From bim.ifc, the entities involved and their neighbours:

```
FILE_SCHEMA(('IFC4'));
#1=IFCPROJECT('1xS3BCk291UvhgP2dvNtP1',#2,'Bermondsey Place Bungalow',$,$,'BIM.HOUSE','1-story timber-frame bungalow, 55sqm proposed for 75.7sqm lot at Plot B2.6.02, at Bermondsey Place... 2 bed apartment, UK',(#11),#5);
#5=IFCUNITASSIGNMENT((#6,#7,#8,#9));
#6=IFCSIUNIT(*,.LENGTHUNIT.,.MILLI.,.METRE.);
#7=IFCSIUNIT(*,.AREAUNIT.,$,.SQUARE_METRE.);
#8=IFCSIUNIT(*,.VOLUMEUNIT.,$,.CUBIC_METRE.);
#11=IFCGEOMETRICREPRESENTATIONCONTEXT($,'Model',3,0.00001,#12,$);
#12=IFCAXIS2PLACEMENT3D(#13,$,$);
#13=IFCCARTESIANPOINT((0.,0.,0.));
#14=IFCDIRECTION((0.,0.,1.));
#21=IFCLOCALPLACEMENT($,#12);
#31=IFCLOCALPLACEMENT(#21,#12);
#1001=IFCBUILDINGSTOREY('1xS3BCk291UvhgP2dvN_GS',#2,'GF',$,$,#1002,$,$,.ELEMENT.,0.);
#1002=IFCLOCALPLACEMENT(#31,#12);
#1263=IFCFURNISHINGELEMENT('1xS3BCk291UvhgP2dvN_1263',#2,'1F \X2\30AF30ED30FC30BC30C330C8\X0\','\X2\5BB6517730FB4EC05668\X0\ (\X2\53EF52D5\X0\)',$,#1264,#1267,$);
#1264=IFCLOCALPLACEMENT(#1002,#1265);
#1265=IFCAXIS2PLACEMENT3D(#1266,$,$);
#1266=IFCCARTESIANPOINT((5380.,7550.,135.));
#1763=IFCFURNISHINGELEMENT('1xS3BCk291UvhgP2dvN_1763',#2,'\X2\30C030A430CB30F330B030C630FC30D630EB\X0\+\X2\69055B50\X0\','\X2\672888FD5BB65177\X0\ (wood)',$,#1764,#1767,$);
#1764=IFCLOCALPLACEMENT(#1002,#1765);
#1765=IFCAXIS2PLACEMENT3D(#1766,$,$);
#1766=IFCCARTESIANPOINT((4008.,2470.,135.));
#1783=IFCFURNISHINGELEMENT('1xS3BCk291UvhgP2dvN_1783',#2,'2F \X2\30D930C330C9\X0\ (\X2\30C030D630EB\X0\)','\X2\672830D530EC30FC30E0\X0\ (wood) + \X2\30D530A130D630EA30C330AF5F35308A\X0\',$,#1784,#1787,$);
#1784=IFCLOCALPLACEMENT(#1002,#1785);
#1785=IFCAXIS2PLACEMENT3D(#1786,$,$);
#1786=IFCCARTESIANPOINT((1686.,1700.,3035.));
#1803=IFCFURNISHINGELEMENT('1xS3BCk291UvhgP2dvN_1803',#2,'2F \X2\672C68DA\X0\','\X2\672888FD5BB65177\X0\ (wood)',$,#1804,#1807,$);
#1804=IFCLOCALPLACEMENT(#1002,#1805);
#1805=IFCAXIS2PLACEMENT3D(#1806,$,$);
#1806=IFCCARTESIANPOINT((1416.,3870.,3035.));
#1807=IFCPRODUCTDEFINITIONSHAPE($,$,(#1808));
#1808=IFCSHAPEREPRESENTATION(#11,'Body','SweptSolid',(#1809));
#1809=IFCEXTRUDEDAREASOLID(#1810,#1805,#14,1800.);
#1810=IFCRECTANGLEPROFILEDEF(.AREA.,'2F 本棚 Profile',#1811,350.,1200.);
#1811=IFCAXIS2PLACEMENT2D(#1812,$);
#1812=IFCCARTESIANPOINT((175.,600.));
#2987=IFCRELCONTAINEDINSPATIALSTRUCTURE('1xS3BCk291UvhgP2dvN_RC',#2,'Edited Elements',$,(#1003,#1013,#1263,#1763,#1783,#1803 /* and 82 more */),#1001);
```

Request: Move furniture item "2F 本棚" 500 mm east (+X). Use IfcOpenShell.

```python
import ifcopenshell
import ifcopenshell.api.geometry
import ifcopenshell.util.placement
import ifcopenshell.util.unit

model = ifcopenshell.open("bim.ifc")
unit_scale = ifcopenshell.util.unit.calculate_unit_scale(model)

item = model.by_id(1803)
matrix = ifcopenshell.util.placement.get_local_placement(item.ObjectPlacement)
matrix[0, 3] += 0.5 / unit_scale
ifcopenshell.api.geometry.edit_object_placement(model, product=item, matrix=matrix, is_si=False)

print(ifcopenshell.util.placement.get_local_placement(item.ObjectPlacement).round(3) + 0.0)

model.write("bim_rev.ifc")
```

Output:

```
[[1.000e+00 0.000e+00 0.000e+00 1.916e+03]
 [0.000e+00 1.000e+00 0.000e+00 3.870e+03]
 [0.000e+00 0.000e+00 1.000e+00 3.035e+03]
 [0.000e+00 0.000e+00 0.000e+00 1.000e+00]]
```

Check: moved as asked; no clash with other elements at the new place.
